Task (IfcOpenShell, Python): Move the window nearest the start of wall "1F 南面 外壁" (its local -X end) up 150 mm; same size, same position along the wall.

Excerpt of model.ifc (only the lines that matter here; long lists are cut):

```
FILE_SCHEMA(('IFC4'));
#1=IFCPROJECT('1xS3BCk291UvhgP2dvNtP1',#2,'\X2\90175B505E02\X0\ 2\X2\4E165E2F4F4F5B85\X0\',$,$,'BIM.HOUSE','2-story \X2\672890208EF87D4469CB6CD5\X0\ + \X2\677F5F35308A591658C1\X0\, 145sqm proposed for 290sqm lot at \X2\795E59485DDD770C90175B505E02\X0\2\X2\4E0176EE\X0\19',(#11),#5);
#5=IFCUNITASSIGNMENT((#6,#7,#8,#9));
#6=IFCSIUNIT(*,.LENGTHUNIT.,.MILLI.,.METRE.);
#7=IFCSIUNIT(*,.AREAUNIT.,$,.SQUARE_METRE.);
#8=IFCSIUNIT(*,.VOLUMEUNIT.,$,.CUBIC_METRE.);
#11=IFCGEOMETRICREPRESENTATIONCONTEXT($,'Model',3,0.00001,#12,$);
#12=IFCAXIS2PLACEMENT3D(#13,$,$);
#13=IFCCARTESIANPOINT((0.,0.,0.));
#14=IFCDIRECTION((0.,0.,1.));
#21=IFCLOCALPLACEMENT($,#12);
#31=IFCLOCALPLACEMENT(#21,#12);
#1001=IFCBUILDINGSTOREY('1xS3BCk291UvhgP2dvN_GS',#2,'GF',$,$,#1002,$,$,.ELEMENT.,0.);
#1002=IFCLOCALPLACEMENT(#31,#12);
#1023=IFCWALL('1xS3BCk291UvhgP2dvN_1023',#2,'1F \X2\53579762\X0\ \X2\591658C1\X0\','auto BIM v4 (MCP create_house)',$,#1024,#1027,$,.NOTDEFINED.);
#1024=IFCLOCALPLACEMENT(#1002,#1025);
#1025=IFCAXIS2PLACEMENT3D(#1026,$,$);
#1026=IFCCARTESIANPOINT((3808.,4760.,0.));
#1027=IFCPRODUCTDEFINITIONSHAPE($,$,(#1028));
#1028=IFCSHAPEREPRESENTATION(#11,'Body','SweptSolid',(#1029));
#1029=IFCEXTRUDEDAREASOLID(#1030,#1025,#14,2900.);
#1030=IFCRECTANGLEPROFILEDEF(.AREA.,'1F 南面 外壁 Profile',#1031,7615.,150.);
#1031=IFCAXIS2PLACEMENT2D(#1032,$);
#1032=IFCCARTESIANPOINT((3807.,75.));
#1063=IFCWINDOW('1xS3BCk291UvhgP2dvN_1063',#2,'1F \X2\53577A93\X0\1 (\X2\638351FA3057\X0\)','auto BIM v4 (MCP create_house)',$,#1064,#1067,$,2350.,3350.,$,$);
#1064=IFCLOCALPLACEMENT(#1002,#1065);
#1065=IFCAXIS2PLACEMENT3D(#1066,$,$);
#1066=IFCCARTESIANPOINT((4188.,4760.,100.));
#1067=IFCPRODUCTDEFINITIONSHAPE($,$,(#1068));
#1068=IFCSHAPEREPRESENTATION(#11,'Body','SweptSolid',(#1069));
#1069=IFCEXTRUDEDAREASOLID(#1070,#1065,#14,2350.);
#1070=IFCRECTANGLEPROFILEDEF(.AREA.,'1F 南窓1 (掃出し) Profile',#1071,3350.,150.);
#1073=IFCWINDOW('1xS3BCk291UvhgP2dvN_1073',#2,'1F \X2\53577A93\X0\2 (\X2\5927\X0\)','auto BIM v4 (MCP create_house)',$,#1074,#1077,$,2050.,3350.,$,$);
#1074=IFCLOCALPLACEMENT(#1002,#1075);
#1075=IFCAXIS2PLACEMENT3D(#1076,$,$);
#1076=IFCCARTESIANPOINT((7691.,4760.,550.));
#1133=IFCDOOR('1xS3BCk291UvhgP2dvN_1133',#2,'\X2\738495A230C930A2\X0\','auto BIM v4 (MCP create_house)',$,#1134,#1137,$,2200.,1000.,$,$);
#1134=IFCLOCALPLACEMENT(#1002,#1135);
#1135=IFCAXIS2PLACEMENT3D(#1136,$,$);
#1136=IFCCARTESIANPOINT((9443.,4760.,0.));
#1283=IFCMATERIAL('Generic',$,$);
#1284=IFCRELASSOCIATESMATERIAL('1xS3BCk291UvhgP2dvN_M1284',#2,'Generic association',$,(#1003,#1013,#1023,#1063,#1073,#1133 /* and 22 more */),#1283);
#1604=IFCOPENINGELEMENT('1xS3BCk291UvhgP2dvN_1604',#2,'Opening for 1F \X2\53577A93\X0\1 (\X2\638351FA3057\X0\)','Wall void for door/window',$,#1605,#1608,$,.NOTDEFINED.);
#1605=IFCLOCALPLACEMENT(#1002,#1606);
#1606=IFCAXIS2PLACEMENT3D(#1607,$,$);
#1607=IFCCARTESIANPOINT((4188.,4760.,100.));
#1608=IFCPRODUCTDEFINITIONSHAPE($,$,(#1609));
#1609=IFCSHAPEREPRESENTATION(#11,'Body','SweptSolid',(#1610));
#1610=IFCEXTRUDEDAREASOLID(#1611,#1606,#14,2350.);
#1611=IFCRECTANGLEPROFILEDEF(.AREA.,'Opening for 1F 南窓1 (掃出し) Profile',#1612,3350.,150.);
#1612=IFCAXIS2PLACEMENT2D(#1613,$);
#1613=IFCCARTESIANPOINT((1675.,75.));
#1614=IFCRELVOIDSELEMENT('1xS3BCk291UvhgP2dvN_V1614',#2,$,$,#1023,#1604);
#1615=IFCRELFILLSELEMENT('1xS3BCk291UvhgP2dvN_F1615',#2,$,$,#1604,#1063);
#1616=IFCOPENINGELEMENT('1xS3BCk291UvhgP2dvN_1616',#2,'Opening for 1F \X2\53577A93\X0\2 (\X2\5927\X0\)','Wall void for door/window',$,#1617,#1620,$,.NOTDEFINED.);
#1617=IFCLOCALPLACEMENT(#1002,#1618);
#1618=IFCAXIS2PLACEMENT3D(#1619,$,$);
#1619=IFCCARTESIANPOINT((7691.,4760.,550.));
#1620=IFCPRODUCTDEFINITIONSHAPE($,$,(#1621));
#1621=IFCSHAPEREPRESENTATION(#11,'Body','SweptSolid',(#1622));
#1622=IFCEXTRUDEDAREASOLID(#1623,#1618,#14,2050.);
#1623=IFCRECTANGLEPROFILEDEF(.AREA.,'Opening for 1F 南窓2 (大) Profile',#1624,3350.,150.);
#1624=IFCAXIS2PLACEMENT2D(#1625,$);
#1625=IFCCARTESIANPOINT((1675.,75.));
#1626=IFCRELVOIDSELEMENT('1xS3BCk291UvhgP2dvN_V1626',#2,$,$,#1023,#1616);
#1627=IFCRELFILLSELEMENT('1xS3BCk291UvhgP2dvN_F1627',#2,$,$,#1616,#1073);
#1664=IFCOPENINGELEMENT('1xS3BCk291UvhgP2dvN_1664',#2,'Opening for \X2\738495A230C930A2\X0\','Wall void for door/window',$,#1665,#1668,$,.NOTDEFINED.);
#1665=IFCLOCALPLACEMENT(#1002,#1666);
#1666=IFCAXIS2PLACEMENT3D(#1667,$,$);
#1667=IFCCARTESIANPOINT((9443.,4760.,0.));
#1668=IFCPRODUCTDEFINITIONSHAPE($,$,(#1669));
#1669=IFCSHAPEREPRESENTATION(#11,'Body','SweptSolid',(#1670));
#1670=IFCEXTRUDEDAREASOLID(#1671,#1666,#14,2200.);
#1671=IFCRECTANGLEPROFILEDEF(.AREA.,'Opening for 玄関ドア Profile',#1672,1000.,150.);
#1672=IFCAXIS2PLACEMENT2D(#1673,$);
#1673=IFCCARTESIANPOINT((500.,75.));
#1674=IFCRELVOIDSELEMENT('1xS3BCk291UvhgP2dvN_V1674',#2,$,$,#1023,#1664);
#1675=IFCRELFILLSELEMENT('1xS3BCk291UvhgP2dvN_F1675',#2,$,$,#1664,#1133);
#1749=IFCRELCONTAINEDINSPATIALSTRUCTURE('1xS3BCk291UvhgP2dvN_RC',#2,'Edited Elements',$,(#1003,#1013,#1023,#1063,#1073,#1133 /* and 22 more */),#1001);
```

```python
import numpy as np
import ifcopenshell
import ifcopenshell.api.geometry
import ifcopenshell.util.placement
import ifcopenshell.util.unit

model = ifcopenshell.open("model.ifc")
unit_scale = ifcopenshell.util.unit.calculate_unit_scale(model)

window = model.by_guid("1xS3BCk291UvhgP2dvN_1063")
opening = window.FillsVoids[0].RelatingOpeningElement
dz = 150.0

shift = np.array([0.0, 0.0, dz])
# The window is not placed relative to its opening, so move both.
for product in (opening, window):
    matrix = ifcopenshell.util.placement.get_local_placement(product.ObjectPlacement)
    matrix[:3, 3] += shift
    ifcopenshell.api.geometry.edit_object_placement(model, product=product, matrix=matrix, is_si=False)

print(f"moved by {dz * unit_scale:+.3f} m")

model.write("model_v2.ifc")
```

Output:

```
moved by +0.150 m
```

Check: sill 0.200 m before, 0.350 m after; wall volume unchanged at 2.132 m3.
